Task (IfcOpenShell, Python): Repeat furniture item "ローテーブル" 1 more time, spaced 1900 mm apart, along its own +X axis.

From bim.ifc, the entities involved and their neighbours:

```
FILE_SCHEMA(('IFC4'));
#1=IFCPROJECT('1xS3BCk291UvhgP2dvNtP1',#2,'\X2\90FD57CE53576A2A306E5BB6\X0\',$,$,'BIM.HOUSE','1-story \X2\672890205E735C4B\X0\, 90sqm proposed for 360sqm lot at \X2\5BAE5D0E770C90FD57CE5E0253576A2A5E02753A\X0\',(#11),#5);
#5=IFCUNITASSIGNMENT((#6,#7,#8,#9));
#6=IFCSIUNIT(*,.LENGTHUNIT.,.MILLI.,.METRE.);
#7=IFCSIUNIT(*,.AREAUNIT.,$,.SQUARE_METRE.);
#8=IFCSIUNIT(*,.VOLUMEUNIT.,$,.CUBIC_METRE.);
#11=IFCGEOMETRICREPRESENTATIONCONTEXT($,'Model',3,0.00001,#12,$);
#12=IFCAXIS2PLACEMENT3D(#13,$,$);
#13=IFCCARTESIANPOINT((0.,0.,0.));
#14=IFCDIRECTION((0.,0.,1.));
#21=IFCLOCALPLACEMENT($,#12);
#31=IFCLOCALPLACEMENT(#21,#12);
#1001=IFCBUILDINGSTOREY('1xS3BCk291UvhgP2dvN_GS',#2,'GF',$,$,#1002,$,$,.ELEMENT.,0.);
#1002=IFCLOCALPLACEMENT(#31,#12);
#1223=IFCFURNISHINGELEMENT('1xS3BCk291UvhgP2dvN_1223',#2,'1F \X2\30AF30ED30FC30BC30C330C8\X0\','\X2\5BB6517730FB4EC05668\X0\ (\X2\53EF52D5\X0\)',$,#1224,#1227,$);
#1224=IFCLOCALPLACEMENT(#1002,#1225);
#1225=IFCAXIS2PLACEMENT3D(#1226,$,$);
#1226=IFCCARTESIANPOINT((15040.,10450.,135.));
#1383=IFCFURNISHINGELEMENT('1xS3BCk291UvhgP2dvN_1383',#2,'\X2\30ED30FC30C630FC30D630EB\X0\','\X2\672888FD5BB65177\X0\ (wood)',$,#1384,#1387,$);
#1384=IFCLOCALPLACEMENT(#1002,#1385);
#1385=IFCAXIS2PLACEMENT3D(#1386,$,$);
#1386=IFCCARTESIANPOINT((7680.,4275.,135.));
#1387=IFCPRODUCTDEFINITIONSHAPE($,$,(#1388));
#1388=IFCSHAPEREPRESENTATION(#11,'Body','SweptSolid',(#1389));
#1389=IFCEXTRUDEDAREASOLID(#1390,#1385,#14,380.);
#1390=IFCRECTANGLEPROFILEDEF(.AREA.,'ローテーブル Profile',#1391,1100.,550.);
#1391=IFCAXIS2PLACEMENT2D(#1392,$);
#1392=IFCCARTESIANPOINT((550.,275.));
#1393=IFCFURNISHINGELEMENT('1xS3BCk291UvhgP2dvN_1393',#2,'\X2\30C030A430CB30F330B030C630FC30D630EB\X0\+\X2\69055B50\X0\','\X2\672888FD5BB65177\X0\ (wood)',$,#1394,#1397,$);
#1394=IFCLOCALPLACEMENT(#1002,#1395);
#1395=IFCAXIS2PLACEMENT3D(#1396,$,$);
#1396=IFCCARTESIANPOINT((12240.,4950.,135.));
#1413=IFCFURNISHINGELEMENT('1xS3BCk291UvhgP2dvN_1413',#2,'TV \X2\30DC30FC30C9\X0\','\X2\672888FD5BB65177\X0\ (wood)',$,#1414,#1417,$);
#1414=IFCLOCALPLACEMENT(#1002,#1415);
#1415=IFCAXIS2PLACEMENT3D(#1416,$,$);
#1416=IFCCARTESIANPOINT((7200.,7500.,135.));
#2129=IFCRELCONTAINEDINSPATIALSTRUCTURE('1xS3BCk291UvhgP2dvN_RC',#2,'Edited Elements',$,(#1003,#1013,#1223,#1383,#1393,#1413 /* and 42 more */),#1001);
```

```python
import ifcopenshell
import ifcopenshell.api.geometry
import ifcopenshell.api.root
import ifcopenshell.util.element
import ifcopenshell.util.placement
import ifcopenshell.util.unit

model = ifcopenshell.open("bim.ifc")
unit_scale = ifcopenshell.util.unit.calculate_unit_scale(model)


def reuse_history(source, copy):
    """copy_class also copies each property set's owner history, people and application; keep the originals."""
    for rel in copy.IsDefinedBy:
        if rel.is_a("IfcRelDefinesByProperties") and (history := rel.RelatingPropertyDefinition.OwnerHistory):
            rel.RelatingPropertyDefinition.OwnerHistory = source.OwnerHistory
            ifcopenshell.util.element.remove_deep2(model, history)


source = model.by_id(1383)
base = ifcopenshell.util.placement.get_local_placement(source.ObjectPlacement)
step = base[:3, 0] * 1.9 / unit_scale

for i in range(1, 2):
    copy = ifcopenshell.api.root.copy_class(model, product=source)
    copy.Representation = ifcopenshell.util.element.copy_deep(
        model, source.Representation, exclude=["IfcGeometricRepresentationContext", "IfcRepresentationMap"]
    )
    reuse_history(source, copy)
    matrix = base.copy()
    matrix[:3, 3] += i * step
    print("added at", matrix[:3, 3].round(3) + 0.0)
    ifcopenshell.api.geometry.edit_object_placement(model, product=copy, matrix=matrix, is_si=False)

model.write("bim_v2.ifc")
```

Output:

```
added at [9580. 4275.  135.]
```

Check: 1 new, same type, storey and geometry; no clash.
